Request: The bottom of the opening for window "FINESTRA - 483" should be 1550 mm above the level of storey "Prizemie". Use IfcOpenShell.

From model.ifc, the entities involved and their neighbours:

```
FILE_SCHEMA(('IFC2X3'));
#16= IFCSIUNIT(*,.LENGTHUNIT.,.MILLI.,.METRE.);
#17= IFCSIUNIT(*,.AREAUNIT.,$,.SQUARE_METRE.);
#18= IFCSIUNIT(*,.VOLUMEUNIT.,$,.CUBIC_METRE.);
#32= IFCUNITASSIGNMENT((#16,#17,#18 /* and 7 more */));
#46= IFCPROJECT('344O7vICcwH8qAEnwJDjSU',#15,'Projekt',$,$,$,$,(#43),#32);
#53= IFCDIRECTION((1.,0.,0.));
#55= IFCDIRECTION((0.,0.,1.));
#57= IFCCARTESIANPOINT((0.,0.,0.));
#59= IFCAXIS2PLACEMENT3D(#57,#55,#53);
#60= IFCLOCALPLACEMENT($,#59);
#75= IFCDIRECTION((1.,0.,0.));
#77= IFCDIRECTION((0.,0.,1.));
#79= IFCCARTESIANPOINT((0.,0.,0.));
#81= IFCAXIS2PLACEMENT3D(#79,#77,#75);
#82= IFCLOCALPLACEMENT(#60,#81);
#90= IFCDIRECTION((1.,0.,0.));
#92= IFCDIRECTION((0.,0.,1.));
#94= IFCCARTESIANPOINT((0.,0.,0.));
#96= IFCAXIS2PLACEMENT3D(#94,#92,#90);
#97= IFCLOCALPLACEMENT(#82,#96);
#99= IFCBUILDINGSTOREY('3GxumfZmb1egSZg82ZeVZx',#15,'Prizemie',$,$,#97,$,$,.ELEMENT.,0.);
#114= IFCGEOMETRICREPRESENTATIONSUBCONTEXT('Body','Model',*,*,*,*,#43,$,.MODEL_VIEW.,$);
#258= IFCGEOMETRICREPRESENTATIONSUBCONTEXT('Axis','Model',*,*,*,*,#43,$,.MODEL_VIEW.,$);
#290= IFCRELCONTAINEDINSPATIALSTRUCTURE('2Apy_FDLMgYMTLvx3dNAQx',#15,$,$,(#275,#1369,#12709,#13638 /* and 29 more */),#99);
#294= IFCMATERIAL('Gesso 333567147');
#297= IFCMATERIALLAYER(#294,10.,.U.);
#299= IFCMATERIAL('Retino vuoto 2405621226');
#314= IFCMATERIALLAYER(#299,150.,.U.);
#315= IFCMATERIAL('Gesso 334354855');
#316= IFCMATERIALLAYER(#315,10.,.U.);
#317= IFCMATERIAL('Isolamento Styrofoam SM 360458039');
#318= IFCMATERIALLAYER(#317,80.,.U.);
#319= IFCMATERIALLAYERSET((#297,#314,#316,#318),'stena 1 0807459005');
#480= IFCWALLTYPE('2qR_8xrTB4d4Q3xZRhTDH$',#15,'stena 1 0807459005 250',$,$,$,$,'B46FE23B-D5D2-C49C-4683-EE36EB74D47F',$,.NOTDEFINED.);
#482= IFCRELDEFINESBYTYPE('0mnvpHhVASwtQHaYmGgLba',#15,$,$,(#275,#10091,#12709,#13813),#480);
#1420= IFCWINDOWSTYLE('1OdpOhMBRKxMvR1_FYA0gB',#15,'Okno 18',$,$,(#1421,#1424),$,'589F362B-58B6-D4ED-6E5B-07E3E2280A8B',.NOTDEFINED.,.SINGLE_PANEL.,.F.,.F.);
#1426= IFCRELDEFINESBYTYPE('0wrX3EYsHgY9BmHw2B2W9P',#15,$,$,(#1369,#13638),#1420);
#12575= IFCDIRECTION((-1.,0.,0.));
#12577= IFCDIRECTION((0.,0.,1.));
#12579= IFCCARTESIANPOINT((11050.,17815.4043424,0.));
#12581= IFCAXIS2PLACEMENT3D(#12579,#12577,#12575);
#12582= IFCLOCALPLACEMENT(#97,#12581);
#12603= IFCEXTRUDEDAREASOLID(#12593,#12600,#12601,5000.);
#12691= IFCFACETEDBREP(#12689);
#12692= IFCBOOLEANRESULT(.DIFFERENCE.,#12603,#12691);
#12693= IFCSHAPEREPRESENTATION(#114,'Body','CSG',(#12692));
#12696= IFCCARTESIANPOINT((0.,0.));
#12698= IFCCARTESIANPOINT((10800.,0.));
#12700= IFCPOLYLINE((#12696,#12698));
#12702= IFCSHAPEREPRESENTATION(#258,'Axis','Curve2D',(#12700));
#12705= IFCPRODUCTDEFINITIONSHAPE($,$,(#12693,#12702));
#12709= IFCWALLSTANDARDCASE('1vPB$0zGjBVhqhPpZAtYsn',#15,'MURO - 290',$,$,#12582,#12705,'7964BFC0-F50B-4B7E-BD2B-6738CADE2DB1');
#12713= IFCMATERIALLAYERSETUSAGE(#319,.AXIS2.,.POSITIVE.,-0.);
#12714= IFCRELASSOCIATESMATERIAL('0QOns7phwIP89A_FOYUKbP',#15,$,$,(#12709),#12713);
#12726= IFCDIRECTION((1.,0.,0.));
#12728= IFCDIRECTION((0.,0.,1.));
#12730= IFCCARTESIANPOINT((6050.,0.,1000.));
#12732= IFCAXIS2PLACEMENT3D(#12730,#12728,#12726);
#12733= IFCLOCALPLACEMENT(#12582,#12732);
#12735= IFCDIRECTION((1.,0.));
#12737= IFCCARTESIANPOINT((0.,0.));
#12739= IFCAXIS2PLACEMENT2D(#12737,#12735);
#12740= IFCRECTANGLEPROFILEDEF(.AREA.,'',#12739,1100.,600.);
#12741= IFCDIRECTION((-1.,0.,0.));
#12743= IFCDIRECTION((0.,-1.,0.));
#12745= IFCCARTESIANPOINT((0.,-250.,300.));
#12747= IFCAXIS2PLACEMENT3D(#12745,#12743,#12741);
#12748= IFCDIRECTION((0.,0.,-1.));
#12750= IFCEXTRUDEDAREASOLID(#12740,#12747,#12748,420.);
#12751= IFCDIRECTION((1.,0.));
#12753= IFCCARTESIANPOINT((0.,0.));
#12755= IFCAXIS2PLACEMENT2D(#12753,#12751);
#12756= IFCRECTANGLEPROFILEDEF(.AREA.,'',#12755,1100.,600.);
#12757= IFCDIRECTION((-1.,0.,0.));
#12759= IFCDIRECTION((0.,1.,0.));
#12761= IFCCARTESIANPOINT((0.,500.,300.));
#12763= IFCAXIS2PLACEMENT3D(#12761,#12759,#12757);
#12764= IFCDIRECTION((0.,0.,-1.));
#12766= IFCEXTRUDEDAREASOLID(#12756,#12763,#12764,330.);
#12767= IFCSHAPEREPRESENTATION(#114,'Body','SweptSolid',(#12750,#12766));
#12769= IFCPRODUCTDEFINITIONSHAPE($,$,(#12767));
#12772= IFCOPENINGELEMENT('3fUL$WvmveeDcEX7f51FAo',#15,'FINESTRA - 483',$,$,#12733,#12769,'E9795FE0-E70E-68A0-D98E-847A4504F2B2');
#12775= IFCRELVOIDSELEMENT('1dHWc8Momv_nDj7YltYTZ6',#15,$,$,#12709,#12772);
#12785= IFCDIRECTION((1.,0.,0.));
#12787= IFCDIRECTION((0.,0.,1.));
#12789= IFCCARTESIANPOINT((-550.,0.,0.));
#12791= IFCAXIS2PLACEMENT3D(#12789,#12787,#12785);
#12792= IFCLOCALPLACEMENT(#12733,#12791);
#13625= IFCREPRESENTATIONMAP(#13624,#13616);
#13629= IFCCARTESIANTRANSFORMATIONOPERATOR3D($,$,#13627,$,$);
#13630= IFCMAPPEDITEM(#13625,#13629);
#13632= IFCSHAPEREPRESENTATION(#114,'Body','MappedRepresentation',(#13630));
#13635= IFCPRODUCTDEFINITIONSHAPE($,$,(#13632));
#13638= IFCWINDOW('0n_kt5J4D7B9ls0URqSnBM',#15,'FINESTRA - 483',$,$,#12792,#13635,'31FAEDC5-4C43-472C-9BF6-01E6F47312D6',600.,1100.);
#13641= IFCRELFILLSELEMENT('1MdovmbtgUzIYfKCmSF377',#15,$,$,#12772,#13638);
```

```python
import numpy as np
import ifcopenshell
import ifcopenshell.api.geometry
import ifcopenshell.geom
import ifcopenshell.util.element
import ifcopenshell.util.placement
import ifcopenshell.util.shape
import ifcopenshell.util.unit

model = ifcopenshell.open("model.ifc")
unit_scale = ifcopenshell.util.unit.calculate_unit_scale(model)

window = model.by_guid("0n_kt5J4D7B9ls0URqSnBM")
opening = window.FillsVoids[0].RelatingOpeningElement
storey = ifcopenshell.util.element.get_container(window, ifc_class="IfcBuildingStorey")
level = ifcopenshell.util.placement.get_local_placement(storey.ObjectPlacement)[2, 3]

# The opening's origin need not be at the sill, so measure its lowest point.
shape = ifcopenshell.geom.create_shape(ifcopenshell.geom.settings(), opening)
bottom = ifcopenshell.util.shape.get_shape_bottom_elevation(shape, shape.geometry) / unit_scale
dz = level + 1550.0 - bottom

shift = np.array([0.0, 0.0, dz])
# The window is placed relative to its opening, so it follows when the opening moves.
matrix = ifcopenshell.util.placement.get_local_placement(opening.ObjectPlacement)
matrix[:3, 3] += shift
ifcopenshell.api.geometry.edit_object_placement(
    model, product=opening, matrix=matrix, is_si=False, should_transform_children=True
)

print(f"moved by {dz * unit_scale:+.3f} m")

model.write("model_updated.ifc")
```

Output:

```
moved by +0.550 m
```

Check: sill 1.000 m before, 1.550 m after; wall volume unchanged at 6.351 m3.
